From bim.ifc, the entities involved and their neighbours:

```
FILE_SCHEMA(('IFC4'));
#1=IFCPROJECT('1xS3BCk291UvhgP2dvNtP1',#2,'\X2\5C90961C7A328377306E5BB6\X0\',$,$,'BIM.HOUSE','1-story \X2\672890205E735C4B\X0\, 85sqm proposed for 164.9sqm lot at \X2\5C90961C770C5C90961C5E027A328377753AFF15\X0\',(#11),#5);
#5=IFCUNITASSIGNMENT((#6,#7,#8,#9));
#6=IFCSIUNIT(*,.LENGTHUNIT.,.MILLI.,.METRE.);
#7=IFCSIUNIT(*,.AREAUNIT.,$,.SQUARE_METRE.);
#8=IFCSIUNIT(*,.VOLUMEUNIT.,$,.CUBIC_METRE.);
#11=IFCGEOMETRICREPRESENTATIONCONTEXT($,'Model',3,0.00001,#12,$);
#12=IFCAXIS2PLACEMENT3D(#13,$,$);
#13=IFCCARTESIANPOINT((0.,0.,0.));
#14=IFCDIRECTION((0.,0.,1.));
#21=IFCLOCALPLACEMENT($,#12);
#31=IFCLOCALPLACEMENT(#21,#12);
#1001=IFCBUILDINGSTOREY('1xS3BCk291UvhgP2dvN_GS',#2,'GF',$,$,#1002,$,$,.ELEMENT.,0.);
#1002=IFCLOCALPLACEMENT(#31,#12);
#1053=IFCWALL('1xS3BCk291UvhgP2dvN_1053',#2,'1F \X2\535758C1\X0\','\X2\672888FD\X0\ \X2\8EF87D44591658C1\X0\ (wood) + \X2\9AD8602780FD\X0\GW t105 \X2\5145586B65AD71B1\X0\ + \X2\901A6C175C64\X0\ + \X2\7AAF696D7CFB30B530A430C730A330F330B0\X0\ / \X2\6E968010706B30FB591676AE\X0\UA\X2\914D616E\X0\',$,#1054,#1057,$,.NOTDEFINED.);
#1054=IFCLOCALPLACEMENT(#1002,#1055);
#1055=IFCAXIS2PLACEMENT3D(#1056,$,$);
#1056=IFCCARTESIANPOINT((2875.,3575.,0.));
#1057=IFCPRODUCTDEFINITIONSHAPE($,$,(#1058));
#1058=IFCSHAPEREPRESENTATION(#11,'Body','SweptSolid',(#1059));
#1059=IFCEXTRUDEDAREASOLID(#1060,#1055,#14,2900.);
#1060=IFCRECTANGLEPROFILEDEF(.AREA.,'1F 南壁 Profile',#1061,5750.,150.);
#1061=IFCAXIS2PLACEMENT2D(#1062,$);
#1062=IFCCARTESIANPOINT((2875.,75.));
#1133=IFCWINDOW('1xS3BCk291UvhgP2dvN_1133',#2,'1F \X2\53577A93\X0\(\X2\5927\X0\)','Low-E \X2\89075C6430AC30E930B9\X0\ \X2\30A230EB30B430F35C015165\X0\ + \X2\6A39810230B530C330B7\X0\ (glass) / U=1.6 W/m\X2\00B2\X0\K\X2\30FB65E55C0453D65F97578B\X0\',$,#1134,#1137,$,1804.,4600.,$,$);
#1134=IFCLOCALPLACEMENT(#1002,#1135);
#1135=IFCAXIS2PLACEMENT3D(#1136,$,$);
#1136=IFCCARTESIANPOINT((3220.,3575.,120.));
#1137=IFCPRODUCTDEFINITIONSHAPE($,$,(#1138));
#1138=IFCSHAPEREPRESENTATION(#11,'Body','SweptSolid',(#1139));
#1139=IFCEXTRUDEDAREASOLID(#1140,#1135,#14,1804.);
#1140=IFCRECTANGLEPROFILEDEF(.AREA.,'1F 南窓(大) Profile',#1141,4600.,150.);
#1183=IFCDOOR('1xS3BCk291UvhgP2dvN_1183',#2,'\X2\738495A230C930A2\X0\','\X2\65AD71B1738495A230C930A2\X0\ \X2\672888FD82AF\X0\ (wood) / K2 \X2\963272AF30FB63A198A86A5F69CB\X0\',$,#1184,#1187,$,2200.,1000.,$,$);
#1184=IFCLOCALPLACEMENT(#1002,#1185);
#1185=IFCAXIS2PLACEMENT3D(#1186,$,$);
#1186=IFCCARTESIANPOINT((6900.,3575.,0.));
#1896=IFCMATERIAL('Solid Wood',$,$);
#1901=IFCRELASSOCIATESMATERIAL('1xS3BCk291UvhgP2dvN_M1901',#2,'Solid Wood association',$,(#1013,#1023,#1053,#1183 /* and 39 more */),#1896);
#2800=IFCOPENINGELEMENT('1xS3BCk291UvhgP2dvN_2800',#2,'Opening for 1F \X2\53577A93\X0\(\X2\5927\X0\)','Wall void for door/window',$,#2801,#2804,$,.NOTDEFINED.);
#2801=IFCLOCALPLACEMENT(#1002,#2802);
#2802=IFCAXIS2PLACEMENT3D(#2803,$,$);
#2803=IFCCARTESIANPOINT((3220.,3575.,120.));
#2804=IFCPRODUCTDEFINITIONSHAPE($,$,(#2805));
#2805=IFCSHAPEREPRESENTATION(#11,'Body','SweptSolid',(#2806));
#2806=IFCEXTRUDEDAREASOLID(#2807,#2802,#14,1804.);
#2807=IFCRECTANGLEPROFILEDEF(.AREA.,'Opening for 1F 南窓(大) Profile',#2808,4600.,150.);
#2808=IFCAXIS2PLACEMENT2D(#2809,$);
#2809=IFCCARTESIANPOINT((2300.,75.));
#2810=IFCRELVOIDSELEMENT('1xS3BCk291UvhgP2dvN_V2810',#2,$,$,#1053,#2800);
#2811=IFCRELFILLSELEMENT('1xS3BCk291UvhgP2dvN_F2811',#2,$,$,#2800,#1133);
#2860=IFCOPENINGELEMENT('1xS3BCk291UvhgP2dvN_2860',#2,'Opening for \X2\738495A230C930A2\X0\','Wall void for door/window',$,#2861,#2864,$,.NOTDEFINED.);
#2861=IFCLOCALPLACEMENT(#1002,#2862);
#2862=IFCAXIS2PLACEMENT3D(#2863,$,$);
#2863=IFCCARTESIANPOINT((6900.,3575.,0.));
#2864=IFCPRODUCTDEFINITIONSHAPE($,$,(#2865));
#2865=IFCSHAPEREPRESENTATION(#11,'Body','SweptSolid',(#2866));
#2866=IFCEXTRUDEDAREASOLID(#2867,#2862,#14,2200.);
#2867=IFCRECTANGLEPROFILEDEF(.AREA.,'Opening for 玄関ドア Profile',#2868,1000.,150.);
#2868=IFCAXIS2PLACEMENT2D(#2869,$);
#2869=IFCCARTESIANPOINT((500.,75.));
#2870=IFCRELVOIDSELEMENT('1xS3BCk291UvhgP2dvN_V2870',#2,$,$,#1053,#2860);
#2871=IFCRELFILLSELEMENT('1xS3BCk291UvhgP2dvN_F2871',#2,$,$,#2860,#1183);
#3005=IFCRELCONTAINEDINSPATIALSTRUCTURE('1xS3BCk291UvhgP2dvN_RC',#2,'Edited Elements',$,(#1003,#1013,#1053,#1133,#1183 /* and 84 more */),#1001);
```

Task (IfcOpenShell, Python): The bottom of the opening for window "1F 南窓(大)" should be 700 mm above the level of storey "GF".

```python
import numpy as np
import ifcopenshell
import ifcopenshell.api.geometry
import ifcopenshell.geom
import ifcopenshell.util.element
import ifcopenshell.util.placement
import ifcopenshell.util.shape
import ifcopenshell.util.unit

model = ifcopenshell.open("bim.ifc")
unit_scale = ifcopenshell.util.unit.calculate_unit_scale(model)

window = model.by_guid("1xS3BCk291UvhgP2dvN_1133")
opening = window.FillsVoids[0].RelatingOpeningElement
storey = ifcopenshell.util.element.get_container(window, ifc_class="IfcBuildingStorey")
level = ifcopenshell.util.placement.get_local_placement(storey.ObjectPlacement)[2, 3]

# The opening's origin need not be at the sill, so measure its lowest point.
shape = ifcopenshell.geom.create_shape(ifcopenshell.geom.settings(), opening)
bottom = ifcopenshell.util.shape.get_shape_bottom_elevation(shape, shape.geometry) / unit_scale
dz = level + 700.0 - bottom

shift = np.array([0.0, 0.0, dz])
# The window is not placed relative to its opening, so move both.
for product in (opening, window):
    matrix = ifcopenshell.util.placement.get_local_placement(product.ObjectPlacement)
    matrix[:3, 3] += shift
    ifcopenshell.api.geometry.edit_object_placement(model, product=product, matrix=matrix, is_si=False)

print(f"moved by {dz * unit_scale:+.3f} m")

model.write("bim_edited.ifc")
```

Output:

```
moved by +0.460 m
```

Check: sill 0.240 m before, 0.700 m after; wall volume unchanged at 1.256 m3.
